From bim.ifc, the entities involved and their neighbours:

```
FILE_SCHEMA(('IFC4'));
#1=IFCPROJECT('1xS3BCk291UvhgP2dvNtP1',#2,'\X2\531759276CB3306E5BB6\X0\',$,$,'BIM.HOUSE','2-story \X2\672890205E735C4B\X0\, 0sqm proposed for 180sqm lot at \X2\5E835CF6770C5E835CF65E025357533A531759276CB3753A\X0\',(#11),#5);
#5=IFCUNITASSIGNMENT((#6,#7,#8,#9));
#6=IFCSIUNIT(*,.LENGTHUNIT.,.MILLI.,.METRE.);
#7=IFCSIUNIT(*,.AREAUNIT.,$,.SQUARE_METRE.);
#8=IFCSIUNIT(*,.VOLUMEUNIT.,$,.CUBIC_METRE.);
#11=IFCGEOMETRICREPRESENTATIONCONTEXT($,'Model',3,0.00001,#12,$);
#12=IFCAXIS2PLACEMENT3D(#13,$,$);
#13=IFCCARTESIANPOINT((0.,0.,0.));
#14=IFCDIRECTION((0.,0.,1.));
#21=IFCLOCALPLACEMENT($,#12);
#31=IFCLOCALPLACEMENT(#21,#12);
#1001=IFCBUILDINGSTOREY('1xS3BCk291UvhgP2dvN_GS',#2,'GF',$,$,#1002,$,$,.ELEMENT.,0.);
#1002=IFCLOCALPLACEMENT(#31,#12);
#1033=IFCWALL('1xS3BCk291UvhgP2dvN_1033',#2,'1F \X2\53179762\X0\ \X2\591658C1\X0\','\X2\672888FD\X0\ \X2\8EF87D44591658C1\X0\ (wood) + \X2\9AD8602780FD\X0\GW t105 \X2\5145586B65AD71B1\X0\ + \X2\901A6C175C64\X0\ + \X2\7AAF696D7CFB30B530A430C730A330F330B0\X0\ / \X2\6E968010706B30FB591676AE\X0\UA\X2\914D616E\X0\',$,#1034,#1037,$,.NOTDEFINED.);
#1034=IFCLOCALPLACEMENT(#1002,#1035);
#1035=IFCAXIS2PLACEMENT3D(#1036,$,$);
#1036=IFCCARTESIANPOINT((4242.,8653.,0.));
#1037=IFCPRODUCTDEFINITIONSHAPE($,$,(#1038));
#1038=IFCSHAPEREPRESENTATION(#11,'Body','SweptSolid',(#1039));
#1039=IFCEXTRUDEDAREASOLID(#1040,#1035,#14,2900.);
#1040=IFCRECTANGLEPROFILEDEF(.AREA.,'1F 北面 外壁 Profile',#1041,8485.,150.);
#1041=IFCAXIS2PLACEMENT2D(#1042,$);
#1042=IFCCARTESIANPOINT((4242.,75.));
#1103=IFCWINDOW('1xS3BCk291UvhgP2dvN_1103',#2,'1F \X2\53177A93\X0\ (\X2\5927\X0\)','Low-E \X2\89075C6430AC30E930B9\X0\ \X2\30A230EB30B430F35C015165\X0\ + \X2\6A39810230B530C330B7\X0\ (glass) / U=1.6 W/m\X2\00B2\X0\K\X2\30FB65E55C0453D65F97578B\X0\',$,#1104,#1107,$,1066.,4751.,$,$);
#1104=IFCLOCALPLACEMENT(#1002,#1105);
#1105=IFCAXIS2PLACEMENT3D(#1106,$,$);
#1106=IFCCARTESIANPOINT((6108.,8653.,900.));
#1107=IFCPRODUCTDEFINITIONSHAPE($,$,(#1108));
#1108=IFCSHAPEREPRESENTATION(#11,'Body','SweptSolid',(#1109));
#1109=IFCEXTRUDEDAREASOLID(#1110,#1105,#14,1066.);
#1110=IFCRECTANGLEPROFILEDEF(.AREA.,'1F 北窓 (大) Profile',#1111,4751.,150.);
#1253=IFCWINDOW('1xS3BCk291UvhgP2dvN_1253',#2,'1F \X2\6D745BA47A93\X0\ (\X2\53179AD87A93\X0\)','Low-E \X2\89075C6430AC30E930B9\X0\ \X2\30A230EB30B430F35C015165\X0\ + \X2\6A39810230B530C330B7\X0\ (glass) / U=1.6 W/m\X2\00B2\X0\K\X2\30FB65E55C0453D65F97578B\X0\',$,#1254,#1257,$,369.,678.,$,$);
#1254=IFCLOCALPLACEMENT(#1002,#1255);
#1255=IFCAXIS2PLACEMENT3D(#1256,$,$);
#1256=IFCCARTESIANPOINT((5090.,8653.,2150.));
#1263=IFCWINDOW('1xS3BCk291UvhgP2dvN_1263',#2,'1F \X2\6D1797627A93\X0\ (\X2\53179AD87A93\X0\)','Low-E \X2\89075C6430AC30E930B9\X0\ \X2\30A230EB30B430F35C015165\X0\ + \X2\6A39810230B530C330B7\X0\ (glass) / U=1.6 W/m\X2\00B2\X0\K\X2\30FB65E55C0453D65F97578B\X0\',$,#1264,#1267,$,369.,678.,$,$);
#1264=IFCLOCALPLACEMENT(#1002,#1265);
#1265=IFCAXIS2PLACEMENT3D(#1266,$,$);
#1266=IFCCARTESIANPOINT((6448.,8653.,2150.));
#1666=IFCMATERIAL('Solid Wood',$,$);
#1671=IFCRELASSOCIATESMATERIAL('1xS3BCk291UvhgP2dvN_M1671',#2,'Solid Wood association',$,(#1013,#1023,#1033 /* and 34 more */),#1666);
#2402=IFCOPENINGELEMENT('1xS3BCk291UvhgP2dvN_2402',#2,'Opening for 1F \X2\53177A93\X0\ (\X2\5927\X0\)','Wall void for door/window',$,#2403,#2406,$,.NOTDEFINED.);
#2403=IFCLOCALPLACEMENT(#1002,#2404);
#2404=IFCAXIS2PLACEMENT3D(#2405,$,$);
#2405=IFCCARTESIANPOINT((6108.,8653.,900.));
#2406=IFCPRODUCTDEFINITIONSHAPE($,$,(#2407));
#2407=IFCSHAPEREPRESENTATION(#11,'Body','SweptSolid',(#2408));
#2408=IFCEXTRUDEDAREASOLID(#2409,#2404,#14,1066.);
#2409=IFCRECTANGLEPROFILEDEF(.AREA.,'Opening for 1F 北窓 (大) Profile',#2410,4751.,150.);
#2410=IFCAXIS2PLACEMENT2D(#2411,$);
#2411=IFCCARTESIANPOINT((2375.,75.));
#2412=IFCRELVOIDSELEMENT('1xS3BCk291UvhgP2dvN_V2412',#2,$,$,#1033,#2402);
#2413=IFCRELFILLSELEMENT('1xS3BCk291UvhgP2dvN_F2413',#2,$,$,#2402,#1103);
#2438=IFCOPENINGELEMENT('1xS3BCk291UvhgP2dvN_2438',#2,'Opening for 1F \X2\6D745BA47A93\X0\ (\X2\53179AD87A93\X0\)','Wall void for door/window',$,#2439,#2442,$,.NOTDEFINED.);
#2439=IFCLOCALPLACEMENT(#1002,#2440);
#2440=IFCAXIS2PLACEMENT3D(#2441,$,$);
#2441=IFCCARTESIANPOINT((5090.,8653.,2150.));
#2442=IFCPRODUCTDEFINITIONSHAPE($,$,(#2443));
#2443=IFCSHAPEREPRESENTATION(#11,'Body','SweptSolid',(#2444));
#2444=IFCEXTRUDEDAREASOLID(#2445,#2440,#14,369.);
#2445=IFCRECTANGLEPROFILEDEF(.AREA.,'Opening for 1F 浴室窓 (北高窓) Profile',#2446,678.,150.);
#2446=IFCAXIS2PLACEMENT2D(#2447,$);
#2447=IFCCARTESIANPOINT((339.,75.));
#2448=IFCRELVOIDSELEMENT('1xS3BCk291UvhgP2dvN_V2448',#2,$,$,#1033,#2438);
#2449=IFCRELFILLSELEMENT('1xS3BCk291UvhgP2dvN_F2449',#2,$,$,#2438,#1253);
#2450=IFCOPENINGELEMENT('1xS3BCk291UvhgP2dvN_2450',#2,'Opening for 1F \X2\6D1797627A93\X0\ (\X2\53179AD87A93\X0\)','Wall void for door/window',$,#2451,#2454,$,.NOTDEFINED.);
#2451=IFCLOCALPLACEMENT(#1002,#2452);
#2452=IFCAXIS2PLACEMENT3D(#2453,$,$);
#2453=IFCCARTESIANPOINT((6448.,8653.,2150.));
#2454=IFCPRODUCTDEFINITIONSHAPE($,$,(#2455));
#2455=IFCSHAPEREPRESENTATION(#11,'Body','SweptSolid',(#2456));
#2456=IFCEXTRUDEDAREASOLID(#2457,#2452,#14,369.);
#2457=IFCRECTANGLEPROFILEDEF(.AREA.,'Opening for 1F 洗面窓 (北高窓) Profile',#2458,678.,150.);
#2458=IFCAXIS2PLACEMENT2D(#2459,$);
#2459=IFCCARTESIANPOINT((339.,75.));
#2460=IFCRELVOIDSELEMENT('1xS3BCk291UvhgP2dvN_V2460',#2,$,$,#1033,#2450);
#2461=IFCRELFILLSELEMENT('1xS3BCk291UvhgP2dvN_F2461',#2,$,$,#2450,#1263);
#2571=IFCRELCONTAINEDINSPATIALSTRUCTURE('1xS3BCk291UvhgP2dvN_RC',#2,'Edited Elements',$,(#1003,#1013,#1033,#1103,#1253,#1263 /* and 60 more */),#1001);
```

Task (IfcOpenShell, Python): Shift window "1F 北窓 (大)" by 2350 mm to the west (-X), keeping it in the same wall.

```python
import ifcopenshell
import ifcopenshell.api.geometry
import ifcopenshell.util.placement
import ifcopenshell.util.unit

model = ifcopenshell.open("bim.ifc")
unit_scale = ifcopenshell.util.unit.calculate_unit_scale(model)

window = model.by_id(1103)
opening = window.FillsVoids[0].RelatingOpeningElement
wall = opening.VoidsElements[0].RelatingBuildingElement

wall_matrix = ifcopenshell.util.placement.get_local_placement(wall.ObjectPlacement)
shift = wall_matrix[:3, 0] * -2.35 / unit_scale
before = ifcopenshell.util.placement.get_local_placement(window.ObjectPlacement)[:3, 3].copy()

# The window is not placed relative to its opening, so move both.
for product in (opening, window):
    matrix = ifcopenshell.util.placement.get_local_placement(product.ObjectPlacement)
    matrix[:3, 3] += shift
    ifcopenshell.api.geometry.edit_object_placement(model, product=product, matrix=matrix, is_si=False)

after = ifcopenshell.util.placement.get_local_placement(window.ObjectPlacement)[:3, 3]
print("window moved by", (after - before).round(3) + 0.0)

model.write("bim_v2.ifc")
```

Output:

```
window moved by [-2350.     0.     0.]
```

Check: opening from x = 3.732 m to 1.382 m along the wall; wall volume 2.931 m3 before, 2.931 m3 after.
